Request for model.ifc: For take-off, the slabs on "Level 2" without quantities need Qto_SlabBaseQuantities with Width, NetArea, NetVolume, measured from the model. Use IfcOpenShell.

First a look at what the model holds.

```python
import ifcopenshell
import ifcopenshell.util.element
import ifcopenshell.util.unit

model = ifcopenshell.open("model.ifc")
print(model.schema)
for unit_type in ("LENGTHUNIT", "AREAUNIT", "VOLUMEUNIT"):
    print(unit_type, ifcopenshell.util.unit.calculate_unit_scale(model, unit_type))
storey = next(s for s in model.by_type("IfcBuildingStorey") if s.Name == "Level 2")
slabs = [e for e in ifcopenshell.util.element.get_decomposition(storey) if e.is_a("IfcSlab")]
for e in sorted(slabs, key=lambda e: e.id()):
    print(e.id(), e.is_a(), e.Name, list(ifcopenshell.util.element.get_psets(e, qtos_only=True)), sep=" | ")
```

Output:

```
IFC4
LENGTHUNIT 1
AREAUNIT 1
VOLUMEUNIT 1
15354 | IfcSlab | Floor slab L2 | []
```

```python
import ifcopenshell
import ifcopenshell.api.pset
import ifcopenshell.geom
import ifcopenshell.util.element
import ifcopenshell.util.shape
import ifcopenshell.util.unit

model = ifcopenshell.open("model.ifc")
unit_scale = ifcopenshell.util.unit.calculate_unit_scale(model)
area_scale = ifcopenshell.util.unit.calculate_unit_scale(model, "AREAUNIT")
volume_scale = ifcopenshell.util.unit.calculate_unit_scale(model, "VOLUMEUNIT")
settings = ifcopenshell.geom.settings()

storey = next(s for s in model.by_type("IfcBuildingStorey") if s.Name == "Level 2")
slabs = [e for e in ifcopenshell.util.element.get_decomposition(storey) if e.is_a("IfcSlab")]

for e in sorted(slabs, key=lambda e: e.id()):
    if ifcopenshell.util.element.get_psets(e, qtos_only=True, should_inherit=False):
        continue
    # Geometry comes back in metres, in the element's own axes.
    shape = ifcopenshell.geom.create_shape(settings, e)
    values = {
        "Width": ifcopenshell.util.shape.get_z(shape.geometry) / unit_scale,
        "NetArea": ifcopenshell.util.shape.get_footprint_area(shape.geometry) / area_scale,
        "NetVolume": ifcopenshell.util.shape.get_volume(shape.geometry) / volume_scale,
    }
    qto = ifcopenshell.api.pset.add_qto(model, product=e, name="Qto_SlabBaseQuantities")
    ifcopenshell.api.pset.edit_qto(model, qto=qto, properties=values)
    print(e.id(), {k: round(v, 3) for k, v in values.items()})

model.write("model_v2.ifc")
```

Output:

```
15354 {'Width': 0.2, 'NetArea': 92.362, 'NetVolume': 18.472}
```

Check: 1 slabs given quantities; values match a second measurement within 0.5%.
